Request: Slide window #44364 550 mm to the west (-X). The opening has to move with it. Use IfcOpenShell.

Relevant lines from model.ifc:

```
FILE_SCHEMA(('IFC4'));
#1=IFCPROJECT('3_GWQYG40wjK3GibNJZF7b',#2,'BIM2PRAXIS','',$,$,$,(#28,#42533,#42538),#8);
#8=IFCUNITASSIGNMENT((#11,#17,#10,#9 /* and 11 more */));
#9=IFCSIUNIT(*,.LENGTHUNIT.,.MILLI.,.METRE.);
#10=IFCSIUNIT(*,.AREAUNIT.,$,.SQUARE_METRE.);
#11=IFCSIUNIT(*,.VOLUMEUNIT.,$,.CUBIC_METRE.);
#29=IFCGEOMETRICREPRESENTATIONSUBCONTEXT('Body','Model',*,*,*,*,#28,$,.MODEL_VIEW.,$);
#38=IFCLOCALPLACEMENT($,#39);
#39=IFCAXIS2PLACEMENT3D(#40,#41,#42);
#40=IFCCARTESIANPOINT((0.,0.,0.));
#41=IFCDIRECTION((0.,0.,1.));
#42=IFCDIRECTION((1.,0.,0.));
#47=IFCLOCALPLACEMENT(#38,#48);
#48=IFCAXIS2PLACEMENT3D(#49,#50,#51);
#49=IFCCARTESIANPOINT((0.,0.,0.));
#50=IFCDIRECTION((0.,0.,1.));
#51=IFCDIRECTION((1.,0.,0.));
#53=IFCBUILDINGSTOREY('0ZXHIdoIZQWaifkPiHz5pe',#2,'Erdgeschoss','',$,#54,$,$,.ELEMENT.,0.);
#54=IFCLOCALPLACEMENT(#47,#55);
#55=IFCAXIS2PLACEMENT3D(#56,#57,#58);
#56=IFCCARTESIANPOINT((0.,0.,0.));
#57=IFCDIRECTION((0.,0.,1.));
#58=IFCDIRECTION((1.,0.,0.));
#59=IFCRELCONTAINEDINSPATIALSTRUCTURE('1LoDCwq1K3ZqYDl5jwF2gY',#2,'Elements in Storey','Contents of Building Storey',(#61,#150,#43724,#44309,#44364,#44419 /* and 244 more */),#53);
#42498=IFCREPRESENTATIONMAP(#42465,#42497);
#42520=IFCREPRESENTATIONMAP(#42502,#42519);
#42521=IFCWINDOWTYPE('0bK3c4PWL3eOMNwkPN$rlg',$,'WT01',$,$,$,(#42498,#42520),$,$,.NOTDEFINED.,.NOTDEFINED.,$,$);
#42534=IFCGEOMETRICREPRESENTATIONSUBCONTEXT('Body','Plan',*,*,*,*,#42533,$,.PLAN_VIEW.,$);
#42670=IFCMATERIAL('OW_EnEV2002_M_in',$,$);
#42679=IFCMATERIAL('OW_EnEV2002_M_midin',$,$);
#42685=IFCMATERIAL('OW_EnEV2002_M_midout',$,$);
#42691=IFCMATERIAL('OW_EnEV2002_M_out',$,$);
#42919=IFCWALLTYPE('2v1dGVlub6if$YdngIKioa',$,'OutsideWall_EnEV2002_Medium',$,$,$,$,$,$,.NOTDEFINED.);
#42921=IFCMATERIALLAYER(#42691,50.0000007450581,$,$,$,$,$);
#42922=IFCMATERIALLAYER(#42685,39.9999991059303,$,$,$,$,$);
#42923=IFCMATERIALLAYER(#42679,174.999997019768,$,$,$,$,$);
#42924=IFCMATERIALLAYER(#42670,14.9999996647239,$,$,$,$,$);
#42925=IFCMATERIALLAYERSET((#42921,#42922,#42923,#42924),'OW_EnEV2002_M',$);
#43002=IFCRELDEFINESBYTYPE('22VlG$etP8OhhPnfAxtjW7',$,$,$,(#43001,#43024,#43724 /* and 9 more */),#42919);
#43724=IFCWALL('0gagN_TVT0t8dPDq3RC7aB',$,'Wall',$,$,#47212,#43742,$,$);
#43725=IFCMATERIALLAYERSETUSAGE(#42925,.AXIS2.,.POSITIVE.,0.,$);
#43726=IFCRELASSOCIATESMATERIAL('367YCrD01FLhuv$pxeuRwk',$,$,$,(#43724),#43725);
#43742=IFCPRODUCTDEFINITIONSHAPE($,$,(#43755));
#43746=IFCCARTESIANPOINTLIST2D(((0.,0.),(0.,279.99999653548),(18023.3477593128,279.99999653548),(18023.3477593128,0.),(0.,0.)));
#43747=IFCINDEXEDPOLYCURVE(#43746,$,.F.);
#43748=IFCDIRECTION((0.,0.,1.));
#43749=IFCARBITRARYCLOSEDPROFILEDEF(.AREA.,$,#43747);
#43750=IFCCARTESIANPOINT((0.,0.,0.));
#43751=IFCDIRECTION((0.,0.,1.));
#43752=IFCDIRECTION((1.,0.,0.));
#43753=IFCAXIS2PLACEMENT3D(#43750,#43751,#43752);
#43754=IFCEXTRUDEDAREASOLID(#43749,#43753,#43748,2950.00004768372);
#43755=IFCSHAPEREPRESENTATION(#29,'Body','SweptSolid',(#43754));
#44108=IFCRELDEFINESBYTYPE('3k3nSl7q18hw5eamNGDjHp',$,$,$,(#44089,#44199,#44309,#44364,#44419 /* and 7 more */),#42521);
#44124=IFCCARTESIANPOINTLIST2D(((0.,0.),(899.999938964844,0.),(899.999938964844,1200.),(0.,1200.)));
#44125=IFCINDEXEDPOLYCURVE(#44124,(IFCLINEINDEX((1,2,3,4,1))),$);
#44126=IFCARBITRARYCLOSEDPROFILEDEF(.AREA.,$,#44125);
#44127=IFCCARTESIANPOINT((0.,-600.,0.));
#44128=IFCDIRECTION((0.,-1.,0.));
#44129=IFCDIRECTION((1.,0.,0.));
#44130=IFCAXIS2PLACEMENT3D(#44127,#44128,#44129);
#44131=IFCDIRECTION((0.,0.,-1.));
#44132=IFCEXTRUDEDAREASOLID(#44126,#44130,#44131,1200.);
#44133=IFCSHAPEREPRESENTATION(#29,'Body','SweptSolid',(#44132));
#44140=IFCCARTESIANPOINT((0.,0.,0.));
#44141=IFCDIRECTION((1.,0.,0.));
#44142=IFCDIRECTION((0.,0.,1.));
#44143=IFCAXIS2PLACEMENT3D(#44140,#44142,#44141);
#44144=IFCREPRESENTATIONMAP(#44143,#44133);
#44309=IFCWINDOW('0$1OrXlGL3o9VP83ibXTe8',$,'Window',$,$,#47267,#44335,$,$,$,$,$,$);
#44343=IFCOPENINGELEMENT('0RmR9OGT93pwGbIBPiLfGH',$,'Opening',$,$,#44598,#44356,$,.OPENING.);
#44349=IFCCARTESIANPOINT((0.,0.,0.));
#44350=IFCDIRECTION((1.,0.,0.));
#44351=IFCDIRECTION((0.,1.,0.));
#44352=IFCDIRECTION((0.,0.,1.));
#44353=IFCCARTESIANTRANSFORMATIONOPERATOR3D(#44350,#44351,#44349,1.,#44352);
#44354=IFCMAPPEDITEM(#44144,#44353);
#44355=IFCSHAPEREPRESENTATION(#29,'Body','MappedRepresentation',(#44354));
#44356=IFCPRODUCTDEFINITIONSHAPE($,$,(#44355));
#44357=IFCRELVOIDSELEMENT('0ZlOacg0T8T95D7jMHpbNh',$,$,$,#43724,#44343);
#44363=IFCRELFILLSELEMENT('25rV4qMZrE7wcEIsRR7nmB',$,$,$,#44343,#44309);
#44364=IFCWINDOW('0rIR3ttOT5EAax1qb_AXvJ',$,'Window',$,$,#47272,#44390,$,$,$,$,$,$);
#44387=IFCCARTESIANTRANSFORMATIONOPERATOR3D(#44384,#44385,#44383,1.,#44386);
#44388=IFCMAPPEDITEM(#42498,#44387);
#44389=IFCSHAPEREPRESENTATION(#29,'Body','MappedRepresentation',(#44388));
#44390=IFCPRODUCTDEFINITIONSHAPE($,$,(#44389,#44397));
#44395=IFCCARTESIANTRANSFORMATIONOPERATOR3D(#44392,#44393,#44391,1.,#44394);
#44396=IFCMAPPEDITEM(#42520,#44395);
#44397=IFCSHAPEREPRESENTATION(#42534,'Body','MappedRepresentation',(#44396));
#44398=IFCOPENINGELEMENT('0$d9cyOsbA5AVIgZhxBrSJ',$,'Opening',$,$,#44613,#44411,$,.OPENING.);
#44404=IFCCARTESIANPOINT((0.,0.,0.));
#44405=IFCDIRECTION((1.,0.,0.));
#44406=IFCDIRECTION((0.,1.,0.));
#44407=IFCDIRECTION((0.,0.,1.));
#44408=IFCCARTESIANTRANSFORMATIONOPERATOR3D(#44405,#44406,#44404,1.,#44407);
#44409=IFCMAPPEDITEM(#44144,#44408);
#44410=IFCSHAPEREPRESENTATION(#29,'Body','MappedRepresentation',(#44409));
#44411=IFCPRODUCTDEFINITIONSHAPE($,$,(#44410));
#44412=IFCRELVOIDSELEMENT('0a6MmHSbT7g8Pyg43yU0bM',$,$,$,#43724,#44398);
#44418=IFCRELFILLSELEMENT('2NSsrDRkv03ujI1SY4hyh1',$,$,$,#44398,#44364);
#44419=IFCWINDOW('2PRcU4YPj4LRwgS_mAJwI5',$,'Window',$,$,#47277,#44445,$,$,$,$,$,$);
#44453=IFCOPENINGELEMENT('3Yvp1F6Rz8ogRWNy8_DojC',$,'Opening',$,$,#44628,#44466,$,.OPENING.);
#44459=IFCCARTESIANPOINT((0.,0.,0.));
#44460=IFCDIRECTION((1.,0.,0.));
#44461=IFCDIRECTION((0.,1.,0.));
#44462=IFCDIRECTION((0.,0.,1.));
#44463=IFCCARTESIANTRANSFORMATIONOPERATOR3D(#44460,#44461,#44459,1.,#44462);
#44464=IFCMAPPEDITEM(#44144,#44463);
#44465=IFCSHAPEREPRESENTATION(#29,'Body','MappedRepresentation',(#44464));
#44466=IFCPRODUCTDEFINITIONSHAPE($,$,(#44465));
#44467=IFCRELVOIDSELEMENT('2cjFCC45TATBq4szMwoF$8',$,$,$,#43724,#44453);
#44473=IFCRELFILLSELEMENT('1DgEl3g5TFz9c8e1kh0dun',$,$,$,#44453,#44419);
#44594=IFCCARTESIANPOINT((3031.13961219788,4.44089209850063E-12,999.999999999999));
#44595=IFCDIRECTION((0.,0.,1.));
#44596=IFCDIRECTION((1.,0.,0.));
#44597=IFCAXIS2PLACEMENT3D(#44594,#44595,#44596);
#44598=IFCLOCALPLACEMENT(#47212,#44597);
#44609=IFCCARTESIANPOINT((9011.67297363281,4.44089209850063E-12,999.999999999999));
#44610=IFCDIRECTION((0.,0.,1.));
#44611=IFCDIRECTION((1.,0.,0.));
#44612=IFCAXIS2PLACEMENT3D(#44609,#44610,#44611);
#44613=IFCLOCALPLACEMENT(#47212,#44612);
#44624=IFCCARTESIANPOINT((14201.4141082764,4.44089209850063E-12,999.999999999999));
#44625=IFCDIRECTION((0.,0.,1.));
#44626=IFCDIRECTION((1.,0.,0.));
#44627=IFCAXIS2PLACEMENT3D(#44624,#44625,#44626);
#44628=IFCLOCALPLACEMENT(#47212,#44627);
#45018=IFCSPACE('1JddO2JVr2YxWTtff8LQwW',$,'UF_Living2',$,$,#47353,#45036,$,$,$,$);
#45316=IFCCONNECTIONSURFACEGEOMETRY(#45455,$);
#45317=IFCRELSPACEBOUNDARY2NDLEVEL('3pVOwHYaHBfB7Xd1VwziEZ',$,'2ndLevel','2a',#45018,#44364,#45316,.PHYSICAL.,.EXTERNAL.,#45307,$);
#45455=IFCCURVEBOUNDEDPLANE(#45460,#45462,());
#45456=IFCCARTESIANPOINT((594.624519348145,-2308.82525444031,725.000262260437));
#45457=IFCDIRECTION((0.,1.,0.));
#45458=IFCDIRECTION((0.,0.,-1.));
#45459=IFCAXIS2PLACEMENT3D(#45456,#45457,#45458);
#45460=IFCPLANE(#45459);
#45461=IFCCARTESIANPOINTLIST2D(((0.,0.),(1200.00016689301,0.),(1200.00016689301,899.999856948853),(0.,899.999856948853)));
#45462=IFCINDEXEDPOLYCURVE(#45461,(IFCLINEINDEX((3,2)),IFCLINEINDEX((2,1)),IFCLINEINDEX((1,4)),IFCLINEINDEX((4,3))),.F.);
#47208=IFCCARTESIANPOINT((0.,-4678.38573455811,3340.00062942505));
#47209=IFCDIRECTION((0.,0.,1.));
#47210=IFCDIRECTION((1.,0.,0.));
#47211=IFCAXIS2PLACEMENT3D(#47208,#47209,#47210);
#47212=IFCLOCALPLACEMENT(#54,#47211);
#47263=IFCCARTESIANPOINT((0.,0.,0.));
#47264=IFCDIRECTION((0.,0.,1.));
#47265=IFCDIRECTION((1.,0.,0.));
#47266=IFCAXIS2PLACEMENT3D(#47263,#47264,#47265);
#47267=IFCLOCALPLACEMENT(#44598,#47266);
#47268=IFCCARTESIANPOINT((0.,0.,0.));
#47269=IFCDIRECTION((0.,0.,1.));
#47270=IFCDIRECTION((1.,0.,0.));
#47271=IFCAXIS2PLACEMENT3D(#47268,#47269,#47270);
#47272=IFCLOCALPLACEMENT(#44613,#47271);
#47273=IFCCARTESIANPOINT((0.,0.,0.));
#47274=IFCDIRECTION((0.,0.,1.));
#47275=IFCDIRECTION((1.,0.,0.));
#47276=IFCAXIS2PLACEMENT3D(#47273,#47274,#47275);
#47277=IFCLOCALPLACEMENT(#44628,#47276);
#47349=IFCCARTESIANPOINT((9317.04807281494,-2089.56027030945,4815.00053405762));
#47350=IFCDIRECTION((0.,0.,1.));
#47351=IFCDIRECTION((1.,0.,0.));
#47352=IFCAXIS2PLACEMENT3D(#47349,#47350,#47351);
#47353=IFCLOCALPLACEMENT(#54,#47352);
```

```python
import numpy as np
import ifcopenshell
import ifcopenshell.api.geometry
import ifcopenshell.util.placement
import ifcopenshell.util.unit

model = ifcopenshell.open("model.ifc")
unit_scale = ifcopenshell.util.unit.calculate_unit_scale(model)

window = model.by_guid("0rIR3ttOT5EAax1qb_AXvJ")
opening = window.FillsVoids[0].RelatingOpeningElement
wall = opening.VoidsElements[0].RelatingBuildingElement

wall_matrix = ifcopenshell.util.placement.get_local_placement(wall.ObjectPlacement)
shift = wall_matrix[:3, 0] * -0.55 / unit_scale
before = ifcopenshell.util.placement.get_local_placement(window.ObjectPlacement)[:3, 3].copy()

# The window is placed relative to its opening, so it follows when the opening moves.
matrix = ifcopenshell.util.placement.get_local_placement(opening.ObjectPlacement)
matrix[:3, 3] += shift
ifcopenshell.api.geometry.edit_object_placement(
    model, product=opening, matrix=matrix, is_si=False, should_transform_children=True
)

# Space boundary surfaces are stored in each space's coordinates; move them too.
for rel in window.ProvidesBoundaries:
    if not rel.ConnectionGeometry:
        continue
    surface = rel.ConnectionGeometry.SurfaceOnRelatingElement.BasisSurface
    space_matrix = ifcopenshell.util.placement.get_local_placement(rel.RelatingSpace.ObjectPlacement)
    point = np.array(surface.Position.Location.Coordinates) + space_matrix[:3, :3].T @ shift
    surface.Position = model.createIfcAxis2Placement3D(
        model.createIfcCartesianPoint(point.tolist()), surface.Position.Axis, surface.Position.RefDirection
    )

after = ifcopenshell.util.placement.get_local_placement(window.ObjectPlacement)[:3, 3]
print("window moved by", (after - before).round(3) + 0.0)

model.write("model_updated.ifc")
```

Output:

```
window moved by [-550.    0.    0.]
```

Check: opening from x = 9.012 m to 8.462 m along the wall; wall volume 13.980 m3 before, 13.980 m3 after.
